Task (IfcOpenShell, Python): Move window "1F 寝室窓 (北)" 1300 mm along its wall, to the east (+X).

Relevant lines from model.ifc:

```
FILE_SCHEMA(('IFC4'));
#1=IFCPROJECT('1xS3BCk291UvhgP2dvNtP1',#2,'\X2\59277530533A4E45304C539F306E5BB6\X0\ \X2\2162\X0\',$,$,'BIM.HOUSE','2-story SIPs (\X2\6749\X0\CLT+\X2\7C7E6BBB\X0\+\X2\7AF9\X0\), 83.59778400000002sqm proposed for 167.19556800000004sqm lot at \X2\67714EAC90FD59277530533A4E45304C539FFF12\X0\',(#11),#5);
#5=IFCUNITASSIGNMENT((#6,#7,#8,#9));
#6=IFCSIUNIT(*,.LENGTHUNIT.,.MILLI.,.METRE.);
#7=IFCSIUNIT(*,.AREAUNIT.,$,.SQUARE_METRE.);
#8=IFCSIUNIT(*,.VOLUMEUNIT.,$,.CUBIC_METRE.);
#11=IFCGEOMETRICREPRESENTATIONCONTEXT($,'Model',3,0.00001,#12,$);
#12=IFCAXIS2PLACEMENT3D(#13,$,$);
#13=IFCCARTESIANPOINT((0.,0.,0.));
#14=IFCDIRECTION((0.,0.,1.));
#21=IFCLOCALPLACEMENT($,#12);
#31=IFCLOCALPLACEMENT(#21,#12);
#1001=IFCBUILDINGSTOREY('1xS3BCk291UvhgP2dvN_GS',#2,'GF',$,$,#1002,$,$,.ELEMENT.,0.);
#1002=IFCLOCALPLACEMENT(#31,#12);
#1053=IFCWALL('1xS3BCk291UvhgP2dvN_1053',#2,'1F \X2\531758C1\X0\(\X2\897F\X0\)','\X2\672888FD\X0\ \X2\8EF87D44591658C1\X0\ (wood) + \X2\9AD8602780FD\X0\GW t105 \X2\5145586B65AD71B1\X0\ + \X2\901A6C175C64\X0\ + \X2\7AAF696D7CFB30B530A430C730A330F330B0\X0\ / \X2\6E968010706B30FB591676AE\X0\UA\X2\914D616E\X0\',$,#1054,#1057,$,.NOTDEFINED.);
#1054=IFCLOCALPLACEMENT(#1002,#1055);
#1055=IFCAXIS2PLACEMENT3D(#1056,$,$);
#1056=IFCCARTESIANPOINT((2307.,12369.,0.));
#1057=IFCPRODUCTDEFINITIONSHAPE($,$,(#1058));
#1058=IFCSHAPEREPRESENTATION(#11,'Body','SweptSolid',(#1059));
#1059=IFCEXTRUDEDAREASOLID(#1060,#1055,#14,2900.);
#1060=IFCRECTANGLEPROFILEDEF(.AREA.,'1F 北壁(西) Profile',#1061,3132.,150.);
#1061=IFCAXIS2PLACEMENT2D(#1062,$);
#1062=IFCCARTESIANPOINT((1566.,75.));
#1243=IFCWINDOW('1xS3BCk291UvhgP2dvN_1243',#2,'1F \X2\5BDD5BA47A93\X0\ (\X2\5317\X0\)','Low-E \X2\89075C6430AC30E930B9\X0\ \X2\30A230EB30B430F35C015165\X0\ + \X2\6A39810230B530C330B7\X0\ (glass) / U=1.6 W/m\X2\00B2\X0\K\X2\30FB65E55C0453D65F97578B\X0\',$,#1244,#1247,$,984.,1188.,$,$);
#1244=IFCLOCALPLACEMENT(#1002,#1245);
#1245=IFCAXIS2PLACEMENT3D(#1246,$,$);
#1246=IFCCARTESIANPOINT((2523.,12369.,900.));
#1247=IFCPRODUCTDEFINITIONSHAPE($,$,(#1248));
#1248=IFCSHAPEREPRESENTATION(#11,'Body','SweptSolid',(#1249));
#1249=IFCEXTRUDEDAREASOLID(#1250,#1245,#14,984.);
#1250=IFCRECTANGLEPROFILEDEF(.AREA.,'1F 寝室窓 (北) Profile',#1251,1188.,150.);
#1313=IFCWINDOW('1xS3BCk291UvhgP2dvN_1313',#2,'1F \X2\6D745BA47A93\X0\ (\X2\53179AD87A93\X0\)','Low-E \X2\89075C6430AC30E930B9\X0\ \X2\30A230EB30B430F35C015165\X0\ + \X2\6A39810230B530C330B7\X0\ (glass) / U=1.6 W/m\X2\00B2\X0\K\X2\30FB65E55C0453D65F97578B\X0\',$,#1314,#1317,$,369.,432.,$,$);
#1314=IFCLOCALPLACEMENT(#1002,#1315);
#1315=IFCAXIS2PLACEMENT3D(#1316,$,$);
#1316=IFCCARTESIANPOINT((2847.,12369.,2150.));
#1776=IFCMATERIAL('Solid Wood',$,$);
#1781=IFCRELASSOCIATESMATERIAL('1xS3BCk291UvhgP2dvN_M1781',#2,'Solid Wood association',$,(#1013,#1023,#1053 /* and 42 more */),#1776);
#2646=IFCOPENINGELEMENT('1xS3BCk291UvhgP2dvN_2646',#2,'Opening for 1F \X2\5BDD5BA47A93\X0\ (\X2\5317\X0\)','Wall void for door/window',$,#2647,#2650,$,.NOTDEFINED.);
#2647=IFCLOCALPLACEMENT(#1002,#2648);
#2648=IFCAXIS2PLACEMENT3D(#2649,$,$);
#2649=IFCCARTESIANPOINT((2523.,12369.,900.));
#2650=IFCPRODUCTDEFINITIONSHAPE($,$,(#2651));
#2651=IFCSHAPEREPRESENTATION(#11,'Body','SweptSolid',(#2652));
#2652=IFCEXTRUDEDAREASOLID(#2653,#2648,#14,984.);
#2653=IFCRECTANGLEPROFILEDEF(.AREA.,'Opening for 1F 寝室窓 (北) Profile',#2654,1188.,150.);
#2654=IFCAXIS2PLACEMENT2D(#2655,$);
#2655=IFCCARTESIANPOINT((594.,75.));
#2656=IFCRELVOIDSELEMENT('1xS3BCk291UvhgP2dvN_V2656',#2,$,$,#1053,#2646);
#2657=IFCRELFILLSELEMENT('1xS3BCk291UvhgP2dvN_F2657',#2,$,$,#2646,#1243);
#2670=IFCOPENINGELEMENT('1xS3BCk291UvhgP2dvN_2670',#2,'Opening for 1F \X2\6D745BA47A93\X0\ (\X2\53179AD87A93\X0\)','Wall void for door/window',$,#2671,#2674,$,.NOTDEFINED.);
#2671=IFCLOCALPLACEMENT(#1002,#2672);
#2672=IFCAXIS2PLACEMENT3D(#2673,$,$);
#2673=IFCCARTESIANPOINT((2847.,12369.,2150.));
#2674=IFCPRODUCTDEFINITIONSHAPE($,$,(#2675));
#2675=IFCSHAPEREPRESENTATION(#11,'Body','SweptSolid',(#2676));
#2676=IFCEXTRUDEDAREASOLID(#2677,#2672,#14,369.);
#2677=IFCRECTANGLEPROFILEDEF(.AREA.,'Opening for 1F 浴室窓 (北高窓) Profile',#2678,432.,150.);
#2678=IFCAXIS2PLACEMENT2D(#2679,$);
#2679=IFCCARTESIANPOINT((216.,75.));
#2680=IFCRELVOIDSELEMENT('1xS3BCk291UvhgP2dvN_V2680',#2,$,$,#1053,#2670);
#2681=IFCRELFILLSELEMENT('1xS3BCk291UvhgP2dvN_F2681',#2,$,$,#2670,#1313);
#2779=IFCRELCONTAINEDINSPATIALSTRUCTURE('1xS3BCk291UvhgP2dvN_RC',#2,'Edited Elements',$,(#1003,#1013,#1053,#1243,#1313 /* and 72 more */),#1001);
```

```python
import ifcopenshell
import ifcopenshell.api.geometry
import ifcopenshell.util.placement
import ifcopenshell.util.unit

model = ifcopenshell.open("model.ifc")
unit_scale = ifcopenshell.util.unit.calculate_unit_scale(model)

window = model.by_guid("1xS3BCk291UvhgP2dvN_1243")
opening = window.FillsVoids[0].RelatingOpeningElement
wall = opening.VoidsElements[0].RelatingBuildingElement

wall_matrix = ifcopenshell.util.placement.get_local_placement(wall.ObjectPlacement)
shift = wall_matrix[:3, 0] * 1.3 / unit_scale
before = ifcopenshell.util.placement.get_local_placement(window.ObjectPlacement)[:3, 3].copy()

# The window is not placed relative to its opening, so move both.
for product in (opening, window):
    matrix = ifcopenshell.util.placement.get_local_placement(product.ObjectPlacement)
    matrix[:3, 3] += shift
    ifcopenshell.api.geometry.edit_object_placement(model, product=product, matrix=matrix, is_si=False)

after = ifcopenshell.util.placement.get_local_placement(window.ObjectPlacement)[:3, 3]
print("window moved by", (after - before).round(3) + 0.0)

model.write("model-out.ifc")
```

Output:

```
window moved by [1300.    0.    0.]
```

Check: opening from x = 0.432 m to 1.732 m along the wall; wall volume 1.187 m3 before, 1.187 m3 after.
